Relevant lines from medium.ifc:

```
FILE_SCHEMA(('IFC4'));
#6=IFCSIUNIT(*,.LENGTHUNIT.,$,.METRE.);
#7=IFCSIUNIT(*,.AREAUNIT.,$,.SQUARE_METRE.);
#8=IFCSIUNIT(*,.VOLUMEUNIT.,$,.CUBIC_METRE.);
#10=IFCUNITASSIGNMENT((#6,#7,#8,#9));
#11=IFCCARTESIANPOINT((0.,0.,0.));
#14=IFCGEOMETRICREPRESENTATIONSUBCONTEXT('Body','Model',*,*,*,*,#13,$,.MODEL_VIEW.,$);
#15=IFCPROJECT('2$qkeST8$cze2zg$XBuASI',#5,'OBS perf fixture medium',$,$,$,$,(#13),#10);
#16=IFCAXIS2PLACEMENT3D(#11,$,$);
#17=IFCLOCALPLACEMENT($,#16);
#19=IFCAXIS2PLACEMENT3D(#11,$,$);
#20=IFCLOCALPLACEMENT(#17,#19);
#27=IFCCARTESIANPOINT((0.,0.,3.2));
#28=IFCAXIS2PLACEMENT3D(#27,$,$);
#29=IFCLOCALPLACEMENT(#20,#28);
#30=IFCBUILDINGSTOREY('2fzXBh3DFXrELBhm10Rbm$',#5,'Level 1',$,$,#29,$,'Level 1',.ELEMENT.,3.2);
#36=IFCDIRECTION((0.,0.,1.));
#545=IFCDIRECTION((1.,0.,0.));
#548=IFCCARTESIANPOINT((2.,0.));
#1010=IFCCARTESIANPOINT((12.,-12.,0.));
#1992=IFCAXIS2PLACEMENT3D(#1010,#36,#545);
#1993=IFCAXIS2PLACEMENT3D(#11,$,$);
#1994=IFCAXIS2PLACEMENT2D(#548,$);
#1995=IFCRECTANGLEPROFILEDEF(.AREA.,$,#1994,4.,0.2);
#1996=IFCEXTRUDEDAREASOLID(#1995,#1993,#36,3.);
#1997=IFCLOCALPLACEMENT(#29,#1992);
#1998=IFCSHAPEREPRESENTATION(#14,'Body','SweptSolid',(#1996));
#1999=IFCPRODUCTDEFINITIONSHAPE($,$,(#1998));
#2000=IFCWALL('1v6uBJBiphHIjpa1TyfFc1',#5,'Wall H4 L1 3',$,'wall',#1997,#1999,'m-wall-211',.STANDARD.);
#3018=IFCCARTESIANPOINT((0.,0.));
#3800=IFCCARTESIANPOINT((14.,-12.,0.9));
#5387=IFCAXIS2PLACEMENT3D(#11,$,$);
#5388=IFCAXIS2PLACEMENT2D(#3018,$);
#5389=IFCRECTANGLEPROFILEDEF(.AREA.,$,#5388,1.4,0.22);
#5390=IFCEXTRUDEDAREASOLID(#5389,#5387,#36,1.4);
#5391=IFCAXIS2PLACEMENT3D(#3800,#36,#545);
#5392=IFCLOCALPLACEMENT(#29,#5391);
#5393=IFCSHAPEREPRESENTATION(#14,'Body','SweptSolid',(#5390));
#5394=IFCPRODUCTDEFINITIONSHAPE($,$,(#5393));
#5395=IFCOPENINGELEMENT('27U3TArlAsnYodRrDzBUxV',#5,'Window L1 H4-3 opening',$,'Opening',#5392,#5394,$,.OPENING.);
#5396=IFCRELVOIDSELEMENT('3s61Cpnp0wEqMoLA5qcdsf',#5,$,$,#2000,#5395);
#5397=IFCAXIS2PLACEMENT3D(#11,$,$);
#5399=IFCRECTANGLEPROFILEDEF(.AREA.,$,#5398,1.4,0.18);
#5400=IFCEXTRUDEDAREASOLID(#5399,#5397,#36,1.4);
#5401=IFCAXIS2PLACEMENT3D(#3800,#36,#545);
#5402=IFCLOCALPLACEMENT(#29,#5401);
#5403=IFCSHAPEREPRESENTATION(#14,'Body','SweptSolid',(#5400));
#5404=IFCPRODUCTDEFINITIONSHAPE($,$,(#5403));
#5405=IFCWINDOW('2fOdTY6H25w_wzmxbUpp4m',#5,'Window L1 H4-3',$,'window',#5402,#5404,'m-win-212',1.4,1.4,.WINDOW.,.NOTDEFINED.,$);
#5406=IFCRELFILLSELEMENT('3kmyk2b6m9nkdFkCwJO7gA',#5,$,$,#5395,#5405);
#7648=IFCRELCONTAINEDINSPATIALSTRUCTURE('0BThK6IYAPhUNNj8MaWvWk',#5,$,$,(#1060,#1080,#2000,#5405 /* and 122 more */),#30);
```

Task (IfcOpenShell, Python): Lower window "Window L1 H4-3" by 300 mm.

```python
import numpy as np
import ifcopenshell
import ifcopenshell.api.geometry
import ifcopenshell.util.placement
import ifcopenshell.util.unit

model = ifcopenshell.open("medium.ifc")
unit_scale = ifcopenshell.util.unit.calculate_unit_scale(model)

window = model.by_id(5405)
opening = window.FillsVoids[0].RelatingOpeningElement
dz = -0.3 / unit_scale

shift = np.array([0.0, 0.0, dz])
# The window is not placed relative to its opening, so move both.
for product in (opening, window):
    matrix = ifcopenshell.util.placement.get_local_placement(product.ObjectPlacement)
    matrix[:3, 3] += shift
    ifcopenshell.api.geometry.edit_object_placement(model, product=product, matrix=matrix, is_si=False)

print(f"moved by {dz * unit_scale:+.3f} m")

model.write("medium_updated.ifc")
```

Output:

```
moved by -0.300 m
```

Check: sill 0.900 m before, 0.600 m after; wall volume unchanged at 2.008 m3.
